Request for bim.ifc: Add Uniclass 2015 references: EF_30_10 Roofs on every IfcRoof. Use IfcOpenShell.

First a look at what the model holds.

```python
import ifcopenshell

model = ifcopenshell.open("bim.ifc")
print(model.schema)
print("classifications:", [c.Name for c in model.by_type("IfcClassification")])
for ifc_class in ("IfcDoor", "IfcRoof", "IfcStair", "IfcWall", "IfcWindow"):
    print(ifc_class, len(model.by_type(ifc_class)))
```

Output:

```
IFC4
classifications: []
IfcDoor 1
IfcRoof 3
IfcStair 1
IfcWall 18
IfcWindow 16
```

```python
import ifcopenshell
import ifcopenshell.api.classification

model = ifcopenshell.open("bim.ifc")

system = ifcopenshell.api.classification.add_classification(model, classification="Uniclass 2015")

codes = {
    "IfcRoof": ("EF_30_10", "Roofs"),
}
for ifc_class, (code, name) in codes.items():
    products = model.by_type(ifc_class)
    ifcopenshell.api.classification.add_reference(
        model, products=products, classification=system, identification=code, name=name
    )
    print(code, len(products))

model.write("bim_edited.ifc")
```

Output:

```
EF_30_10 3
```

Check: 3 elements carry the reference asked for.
